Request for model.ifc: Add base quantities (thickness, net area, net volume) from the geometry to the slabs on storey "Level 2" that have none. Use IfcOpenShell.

First a look at what the model holds.

```python
import ifcopenshell
import ifcopenshell.util.element
import ifcopenshell.util.unit

model = ifcopenshell.open("model.ifc")
print(model.schema)
for unit_type in ("LENGTHUNIT", "AREAUNIT", "VOLUMEUNIT"):
    print(unit_type, ifcopenshell.util.unit.calculate_unit_scale(model, unit_type))
storey = next(s for s in model.by_type("IfcBuildingStorey") if s.Name == "Level 2")
slabs = [e for e in ifcopenshell.util.element.get_decomposition(storey) if e.is_a("IfcSlab")]
for e in sorted(slabs, key=lambda e: e.id()):
    print(e.id(), e.is_a(), e.Name, list(ifcopenshell.util.element.get_psets(e, qtos_only=True)), sep=" | ")
```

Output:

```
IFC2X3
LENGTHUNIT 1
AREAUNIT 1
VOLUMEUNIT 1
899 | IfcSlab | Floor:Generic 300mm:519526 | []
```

```python
import ifcopenshell
import ifcopenshell.api.pset
import ifcopenshell.geom
import ifcopenshell.util.element
import ifcopenshell.util.shape
import ifcopenshell.util.unit

model = ifcopenshell.open("model.ifc")
unit_scale = ifcopenshell.util.unit.calculate_unit_scale(model)
area_scale = ifcopenshell.util.unit.calculate_unit_scale(model, "AREAUNIT")
volume_scale = ifcopenshell.util.unit.calculate_unit_scale(model, "VOLUMEUNIT")
settings = ifcopenshell.geom.settings()

storey = next(s for s in model.by_type("IfcBuildingStorey") if s.Name == "Level 2")
slabs = [e for e in ifcopenshell.util.element.get_decomposition(storey) if e.is_a("IfcSlab")]

for e in sorted(slabs, key=lambda e: e.id()):
    if ifcopenshell.util.element.get_psets(e, qtos_only=True, should_inherit=False):
        continue
    # Geometry comes back in metres, in the element's own axes.
    shape = ifcopenshell.geom.create_shape(settings, e)
    values = {
        "Width": ifcopenshell.util.shape.get_z(shape.geometry) / unit_scale,
        "NetArea": ifcopenshell.util.shape.get_footprint_area(shape.geometry) / area_scale,
        "NetVolume": ifcopenshell.util.shape.get_volume(shape.geometry) / volume_scale,
    }
    qto = ifcopenshell.api.pset.add_qto(model, product=e, name="BaseQuantities")
    ifcopenshell.api.pset.edit_qto(model, qto=qto, properties=values)
    print(e.id(), {k: round(v, 3) for k, v in values.items()})

model.write("model_rev.ifc")
```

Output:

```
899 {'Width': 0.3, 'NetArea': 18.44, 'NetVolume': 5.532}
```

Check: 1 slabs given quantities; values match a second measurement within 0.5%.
